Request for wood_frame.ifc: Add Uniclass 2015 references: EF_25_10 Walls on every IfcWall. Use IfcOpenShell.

First a look at what the model holds.

```python
import ifcopenshell

model = ifcopenshell.open("wood_frame.ifc")
print(model.schema)
print("classifications:", [c.Name for c in model.by_type("IfcClassification")])
for ifc_class in ("IfcDoor", "IfcRoof", "IfcStair", "IfcWall", "IfcWindow"):
    print(ifc_class, len(model.by_type(ifc_class)))
```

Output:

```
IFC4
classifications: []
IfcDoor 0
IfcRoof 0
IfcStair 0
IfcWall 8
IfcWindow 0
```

```python
import ifcopenshell
import ifcopenshell.api.classification

model = ifcopenshell.open("wood_frame.ifc")

system = ifcopenshell.api.classification.add_classification(model, classification="Uniclass 2015")

codes = {
    "IfcWall": ("EF_25_10", "Walls"),
}
for ifc_class, (code, name) in codes.items():
    products = model.by_type(ifc_class)
    ifcopenshell.api.classification.add_reference(
        model, products=products, classification=system, identification=code, name=name
    )
    print(code, len(products))

model.write("wood_frame_rev.ifc")
```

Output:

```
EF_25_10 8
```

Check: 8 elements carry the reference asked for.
